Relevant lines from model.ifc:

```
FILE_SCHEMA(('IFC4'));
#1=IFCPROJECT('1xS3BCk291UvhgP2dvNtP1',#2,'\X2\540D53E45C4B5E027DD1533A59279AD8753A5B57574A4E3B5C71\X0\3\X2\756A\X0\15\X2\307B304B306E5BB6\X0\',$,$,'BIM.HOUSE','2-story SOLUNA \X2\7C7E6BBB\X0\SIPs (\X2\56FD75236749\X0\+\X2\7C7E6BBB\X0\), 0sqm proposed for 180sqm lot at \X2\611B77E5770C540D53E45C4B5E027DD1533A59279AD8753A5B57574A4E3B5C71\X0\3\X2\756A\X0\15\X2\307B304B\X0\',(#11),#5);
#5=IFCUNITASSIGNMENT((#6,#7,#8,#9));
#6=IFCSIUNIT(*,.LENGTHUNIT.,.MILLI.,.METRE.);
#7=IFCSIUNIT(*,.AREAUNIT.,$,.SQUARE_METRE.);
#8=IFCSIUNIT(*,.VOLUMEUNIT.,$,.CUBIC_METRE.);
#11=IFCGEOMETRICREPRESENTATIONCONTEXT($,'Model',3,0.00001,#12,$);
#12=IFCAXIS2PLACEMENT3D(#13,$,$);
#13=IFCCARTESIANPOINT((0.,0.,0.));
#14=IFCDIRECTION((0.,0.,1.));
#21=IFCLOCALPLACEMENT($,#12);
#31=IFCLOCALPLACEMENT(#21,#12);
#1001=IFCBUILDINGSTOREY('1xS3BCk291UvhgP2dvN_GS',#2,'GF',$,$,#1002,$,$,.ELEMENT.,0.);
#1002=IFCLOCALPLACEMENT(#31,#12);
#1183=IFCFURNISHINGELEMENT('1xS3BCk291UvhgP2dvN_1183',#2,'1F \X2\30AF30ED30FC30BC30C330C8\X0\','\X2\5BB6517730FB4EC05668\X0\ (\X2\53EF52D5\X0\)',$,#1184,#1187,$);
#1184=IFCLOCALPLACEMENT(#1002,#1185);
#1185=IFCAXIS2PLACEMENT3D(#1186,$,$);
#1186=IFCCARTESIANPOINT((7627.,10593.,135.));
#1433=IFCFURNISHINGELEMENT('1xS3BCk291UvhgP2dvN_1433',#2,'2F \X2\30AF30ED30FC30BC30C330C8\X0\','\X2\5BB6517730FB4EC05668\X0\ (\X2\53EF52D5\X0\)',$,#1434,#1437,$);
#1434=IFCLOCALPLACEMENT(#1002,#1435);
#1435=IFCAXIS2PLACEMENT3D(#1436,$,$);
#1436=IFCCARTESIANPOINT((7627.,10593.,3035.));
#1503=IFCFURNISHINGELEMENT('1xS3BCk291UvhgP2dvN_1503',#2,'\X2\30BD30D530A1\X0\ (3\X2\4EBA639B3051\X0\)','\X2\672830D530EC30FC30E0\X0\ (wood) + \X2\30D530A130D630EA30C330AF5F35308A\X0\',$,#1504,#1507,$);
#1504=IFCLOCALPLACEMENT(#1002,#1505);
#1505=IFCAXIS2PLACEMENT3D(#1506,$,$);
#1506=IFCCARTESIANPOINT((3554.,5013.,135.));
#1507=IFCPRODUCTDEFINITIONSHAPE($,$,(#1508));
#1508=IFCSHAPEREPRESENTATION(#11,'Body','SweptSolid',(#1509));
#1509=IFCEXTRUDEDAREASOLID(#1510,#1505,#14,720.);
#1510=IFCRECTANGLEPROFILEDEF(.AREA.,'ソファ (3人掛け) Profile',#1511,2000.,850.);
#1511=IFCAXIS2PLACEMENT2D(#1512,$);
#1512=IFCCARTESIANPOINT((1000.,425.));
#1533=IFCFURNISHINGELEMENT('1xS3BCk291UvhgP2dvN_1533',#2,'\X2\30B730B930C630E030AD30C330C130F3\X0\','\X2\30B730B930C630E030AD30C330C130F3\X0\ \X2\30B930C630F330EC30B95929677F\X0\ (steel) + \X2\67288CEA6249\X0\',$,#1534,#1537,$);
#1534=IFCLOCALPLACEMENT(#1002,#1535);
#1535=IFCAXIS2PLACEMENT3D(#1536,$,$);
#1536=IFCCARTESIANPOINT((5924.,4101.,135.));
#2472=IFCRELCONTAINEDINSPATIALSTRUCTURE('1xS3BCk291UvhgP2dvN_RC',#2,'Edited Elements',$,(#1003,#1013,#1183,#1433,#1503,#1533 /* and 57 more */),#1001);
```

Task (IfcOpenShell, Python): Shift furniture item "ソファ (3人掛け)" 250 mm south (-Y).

```python
import ifcopenshell
import ifcopenshell.api.geometry
import ifcopenshell.util.placement
import ifcopenshell.util.unit

model = ifcopenshell.open("model.ifc")
unit_scale = ifcopenshell.util.unit.calculate_unit_scale(model)

item = model.by_id(1503)
matrix = ifcopenshell.util.placement.get_local_placement(item.ObjectPlacement)
matrix[1, 3] -= 0.25 / unit_scale
ifcopenshell.api.geometry.edit_object_placement(model, product=item, matrix=matrix, is_si=False)

print(ifcopenshell.util.placement.get_local_placement(item.ObjectPlacement).round(3) + 0.0)

model.write("model-out.ifc")
```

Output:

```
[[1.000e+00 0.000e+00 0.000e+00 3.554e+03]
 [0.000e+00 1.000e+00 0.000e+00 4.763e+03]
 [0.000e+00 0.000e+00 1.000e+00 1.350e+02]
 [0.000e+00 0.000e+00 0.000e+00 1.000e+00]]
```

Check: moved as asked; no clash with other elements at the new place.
